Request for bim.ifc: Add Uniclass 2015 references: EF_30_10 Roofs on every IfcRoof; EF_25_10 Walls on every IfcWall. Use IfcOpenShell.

First a look at what the model holds.

```python
import ifcopenshell

model = ifcopenshell.open("bim.ifc")
print(model.schema)
print("classifications:", [c.Name for c in model.by_type("IfcClassification")])
for ifc_class in ("IfcDoor", "IfcRoof", "IfcStair", "IfcWall", "IfcWindow"):
    print(ifc_class, len(model.by_type(ifc_class)))
```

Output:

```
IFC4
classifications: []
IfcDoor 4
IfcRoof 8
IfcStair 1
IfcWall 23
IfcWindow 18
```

```python
import ifcopenshell
import ifcopenshell.api.classification

model = ifcopenshell.open("bim.ifc")

system = ifcopenshell.api.classification.add_classification(model, classification="Uniclass 2015")

codes = {
    "IfcRoof": ("EF_30_10", "Roofs"),
    "IfcWall": ("EF_25_10", "Walls"),
}
for ifc_class, (code, name) in codes.items():
    products = model.by_type(ifc_class)
    ifcopenshell.api.classification.add_reference(
        model, products=products, classification=system, identification=code, name=name
    )
    print(code, len(products))

model.write("bim-out.ifc")
```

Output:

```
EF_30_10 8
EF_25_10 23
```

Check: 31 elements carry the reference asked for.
